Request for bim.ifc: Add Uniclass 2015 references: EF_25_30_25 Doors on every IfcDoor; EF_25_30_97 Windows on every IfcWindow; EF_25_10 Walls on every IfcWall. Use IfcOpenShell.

First a look at what the model holds.

```python
import ifcopenshell

model = ifcopenshell.open("bim.ifc")
print(model.schema)
print("classifications:", [c.Name for c in model.by_type("IfcClassification")])
for ifc_class in ("IfcDoor", "IfcRoof", "IfcStair", "IfcWall", "IfcWindow"):
    print(ifc_class, len(model.by_type(ifc_class)))
```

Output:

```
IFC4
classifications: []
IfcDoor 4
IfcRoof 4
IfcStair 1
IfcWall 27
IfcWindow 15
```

```python
import ifcopenshell
import ifcopenshell.api.classification

model = ifcopenshell.open("bim.ifc")

system = ifcopenshell.api.classification.add_classification(model, classification="Uniclass 2015")

codes = {
    "IfcDoor": ("EF_25_30_25", "Doors"),
    "IfcWindow": ("EF_25_30_97", "Windows"),
    "IfcWall": ("EF_25_10", "Walls"),
}
for ifc_class, (code, name) in codes.items():
    products = model.by_type(ifc_class)
    ifcopenshell.api.classification.add_reference(
        model, products=products, classification=system, identification=code, name=name
    )
    print(code, len(products))

model.write("bim_v2.ifc")
```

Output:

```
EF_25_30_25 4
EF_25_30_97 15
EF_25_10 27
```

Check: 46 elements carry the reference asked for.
